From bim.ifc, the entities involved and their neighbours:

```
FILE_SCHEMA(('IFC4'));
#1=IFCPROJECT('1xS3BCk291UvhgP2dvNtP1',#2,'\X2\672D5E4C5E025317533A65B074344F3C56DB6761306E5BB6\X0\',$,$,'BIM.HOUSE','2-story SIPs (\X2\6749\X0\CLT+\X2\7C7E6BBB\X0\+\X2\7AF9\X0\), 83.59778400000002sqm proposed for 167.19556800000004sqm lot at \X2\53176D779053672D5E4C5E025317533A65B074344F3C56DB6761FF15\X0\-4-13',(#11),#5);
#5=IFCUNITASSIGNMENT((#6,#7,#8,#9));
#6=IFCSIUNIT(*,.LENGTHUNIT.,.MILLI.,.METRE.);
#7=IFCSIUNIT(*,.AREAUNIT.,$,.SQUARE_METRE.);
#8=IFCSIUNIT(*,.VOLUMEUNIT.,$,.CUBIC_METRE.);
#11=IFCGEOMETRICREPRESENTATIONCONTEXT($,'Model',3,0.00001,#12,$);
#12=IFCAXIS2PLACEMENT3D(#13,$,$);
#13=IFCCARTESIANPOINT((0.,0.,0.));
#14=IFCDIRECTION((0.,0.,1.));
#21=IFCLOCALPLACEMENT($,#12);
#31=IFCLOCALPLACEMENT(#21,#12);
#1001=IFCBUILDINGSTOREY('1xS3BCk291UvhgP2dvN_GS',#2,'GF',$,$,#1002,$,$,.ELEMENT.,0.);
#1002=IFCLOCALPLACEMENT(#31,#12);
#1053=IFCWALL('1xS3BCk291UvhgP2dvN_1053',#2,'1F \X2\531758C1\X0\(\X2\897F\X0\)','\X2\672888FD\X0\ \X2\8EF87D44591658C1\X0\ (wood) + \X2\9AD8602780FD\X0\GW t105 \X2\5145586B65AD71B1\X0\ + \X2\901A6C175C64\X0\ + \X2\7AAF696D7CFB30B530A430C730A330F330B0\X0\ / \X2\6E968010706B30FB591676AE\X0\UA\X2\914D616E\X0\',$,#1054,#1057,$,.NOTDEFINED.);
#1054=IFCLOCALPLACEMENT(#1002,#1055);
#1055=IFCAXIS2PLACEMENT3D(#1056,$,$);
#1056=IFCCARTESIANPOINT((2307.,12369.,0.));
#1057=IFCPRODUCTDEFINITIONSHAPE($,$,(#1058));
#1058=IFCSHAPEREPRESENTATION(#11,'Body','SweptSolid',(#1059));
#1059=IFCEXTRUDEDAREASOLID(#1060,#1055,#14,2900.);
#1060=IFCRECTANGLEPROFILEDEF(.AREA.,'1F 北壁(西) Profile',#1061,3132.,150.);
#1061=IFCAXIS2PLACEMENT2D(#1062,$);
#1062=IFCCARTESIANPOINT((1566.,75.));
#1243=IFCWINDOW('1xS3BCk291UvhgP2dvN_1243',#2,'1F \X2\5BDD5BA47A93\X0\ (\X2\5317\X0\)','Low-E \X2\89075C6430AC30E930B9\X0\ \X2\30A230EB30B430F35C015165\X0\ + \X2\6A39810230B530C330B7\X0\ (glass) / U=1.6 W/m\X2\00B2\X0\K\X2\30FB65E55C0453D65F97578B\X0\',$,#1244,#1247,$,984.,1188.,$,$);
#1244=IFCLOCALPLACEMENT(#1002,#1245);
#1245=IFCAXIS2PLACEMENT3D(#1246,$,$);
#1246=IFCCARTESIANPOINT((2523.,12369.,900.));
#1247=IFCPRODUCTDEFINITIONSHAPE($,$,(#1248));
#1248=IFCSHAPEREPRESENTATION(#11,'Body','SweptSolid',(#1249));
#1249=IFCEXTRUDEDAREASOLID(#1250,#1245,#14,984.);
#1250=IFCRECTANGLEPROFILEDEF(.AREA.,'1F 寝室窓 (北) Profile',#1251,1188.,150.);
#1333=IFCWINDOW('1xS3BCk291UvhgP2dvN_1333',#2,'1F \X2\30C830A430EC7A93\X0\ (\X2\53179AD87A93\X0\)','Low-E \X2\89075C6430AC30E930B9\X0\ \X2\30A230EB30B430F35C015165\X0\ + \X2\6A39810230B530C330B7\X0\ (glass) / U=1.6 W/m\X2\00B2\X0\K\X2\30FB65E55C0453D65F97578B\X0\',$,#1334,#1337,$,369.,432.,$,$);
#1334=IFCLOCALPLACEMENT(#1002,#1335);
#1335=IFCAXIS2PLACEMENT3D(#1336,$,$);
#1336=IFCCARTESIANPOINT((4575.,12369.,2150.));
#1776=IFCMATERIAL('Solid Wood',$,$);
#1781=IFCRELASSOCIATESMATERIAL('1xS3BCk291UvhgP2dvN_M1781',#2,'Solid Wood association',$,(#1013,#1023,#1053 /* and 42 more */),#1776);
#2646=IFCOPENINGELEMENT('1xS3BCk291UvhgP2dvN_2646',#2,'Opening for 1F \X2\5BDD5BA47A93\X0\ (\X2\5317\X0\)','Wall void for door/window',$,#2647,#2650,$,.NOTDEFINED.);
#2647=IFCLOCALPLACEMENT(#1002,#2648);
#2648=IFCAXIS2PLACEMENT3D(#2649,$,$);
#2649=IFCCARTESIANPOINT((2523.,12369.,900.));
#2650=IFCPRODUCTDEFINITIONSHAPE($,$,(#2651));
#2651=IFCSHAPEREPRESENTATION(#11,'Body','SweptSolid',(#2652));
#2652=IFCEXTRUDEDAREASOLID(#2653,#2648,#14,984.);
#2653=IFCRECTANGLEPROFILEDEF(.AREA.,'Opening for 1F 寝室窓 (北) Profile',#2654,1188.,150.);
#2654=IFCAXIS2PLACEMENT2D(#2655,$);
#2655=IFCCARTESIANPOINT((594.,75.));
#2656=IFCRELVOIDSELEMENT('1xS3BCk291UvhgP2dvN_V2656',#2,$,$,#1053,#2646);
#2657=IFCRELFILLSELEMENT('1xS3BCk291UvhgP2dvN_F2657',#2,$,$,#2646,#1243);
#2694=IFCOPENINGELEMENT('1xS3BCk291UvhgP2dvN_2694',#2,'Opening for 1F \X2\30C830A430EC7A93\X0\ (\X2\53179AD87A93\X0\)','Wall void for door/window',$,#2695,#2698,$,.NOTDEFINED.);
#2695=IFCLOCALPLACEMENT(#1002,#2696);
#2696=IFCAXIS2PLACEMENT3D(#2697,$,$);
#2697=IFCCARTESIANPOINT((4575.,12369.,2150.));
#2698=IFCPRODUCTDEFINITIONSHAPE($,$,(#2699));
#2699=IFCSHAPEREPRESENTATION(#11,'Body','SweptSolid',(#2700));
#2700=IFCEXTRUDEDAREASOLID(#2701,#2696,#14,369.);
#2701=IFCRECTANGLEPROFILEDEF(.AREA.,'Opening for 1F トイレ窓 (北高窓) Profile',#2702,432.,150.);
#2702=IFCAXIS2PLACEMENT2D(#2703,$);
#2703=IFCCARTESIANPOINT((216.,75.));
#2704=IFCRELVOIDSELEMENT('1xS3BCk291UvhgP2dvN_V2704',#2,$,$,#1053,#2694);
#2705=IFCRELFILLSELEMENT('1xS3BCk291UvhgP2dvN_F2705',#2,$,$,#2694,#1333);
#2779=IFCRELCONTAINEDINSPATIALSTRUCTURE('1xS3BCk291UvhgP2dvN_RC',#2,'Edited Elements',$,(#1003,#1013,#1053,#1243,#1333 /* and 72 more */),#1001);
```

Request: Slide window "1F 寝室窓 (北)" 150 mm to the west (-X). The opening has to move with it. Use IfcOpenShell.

```python
import ifcopenshell
import ifcopenshell.api.geometry
import ifcopenshell.util.placement
import ifcopenshell.util.unit

model = ifcopenshell.open("bim.ifc")
unit_scale = ifcopenshell.util.unit.calculate_unit_scale(model)

window = model.by_guid("1xS3BCk291UvhgP2dvN_1243")
opening = window.FillsVoids[0].RelatingOpeningElement
wall = opening.VoidsElements[0].RelatingBuildingElement

wall_matrix = ifcopenshell.util.placement.get_local_placement(wall.ObjectPlacement)
shift = wall_matrix[:3, 0] * -0.15 / unit_scale
before = ifcopenshell.util.placement.get_local_placement(window.ObjectPlacement)[:3, 3].copy()

# The window is not placed relative to its opening, so move both.
for product in (opening, window):
    matrix = ifcopenshell.util.placement.get_local_placement(product.ObjectPlacement)
    matrix[:3, 3] += shift
    ifcopenshell.api.geometry.edit_object_placement(model, product=product, matrix=matrix, is_si=False)

after = ifcopenshell.util.placement.get_local_placement(window.ObjectPlacement)[:3, 3]
print("window moved by", (after - before).round(3) + 0.0)

model.write("bim_v2.ifc")
```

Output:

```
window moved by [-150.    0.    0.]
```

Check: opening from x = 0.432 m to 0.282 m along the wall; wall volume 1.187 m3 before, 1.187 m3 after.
